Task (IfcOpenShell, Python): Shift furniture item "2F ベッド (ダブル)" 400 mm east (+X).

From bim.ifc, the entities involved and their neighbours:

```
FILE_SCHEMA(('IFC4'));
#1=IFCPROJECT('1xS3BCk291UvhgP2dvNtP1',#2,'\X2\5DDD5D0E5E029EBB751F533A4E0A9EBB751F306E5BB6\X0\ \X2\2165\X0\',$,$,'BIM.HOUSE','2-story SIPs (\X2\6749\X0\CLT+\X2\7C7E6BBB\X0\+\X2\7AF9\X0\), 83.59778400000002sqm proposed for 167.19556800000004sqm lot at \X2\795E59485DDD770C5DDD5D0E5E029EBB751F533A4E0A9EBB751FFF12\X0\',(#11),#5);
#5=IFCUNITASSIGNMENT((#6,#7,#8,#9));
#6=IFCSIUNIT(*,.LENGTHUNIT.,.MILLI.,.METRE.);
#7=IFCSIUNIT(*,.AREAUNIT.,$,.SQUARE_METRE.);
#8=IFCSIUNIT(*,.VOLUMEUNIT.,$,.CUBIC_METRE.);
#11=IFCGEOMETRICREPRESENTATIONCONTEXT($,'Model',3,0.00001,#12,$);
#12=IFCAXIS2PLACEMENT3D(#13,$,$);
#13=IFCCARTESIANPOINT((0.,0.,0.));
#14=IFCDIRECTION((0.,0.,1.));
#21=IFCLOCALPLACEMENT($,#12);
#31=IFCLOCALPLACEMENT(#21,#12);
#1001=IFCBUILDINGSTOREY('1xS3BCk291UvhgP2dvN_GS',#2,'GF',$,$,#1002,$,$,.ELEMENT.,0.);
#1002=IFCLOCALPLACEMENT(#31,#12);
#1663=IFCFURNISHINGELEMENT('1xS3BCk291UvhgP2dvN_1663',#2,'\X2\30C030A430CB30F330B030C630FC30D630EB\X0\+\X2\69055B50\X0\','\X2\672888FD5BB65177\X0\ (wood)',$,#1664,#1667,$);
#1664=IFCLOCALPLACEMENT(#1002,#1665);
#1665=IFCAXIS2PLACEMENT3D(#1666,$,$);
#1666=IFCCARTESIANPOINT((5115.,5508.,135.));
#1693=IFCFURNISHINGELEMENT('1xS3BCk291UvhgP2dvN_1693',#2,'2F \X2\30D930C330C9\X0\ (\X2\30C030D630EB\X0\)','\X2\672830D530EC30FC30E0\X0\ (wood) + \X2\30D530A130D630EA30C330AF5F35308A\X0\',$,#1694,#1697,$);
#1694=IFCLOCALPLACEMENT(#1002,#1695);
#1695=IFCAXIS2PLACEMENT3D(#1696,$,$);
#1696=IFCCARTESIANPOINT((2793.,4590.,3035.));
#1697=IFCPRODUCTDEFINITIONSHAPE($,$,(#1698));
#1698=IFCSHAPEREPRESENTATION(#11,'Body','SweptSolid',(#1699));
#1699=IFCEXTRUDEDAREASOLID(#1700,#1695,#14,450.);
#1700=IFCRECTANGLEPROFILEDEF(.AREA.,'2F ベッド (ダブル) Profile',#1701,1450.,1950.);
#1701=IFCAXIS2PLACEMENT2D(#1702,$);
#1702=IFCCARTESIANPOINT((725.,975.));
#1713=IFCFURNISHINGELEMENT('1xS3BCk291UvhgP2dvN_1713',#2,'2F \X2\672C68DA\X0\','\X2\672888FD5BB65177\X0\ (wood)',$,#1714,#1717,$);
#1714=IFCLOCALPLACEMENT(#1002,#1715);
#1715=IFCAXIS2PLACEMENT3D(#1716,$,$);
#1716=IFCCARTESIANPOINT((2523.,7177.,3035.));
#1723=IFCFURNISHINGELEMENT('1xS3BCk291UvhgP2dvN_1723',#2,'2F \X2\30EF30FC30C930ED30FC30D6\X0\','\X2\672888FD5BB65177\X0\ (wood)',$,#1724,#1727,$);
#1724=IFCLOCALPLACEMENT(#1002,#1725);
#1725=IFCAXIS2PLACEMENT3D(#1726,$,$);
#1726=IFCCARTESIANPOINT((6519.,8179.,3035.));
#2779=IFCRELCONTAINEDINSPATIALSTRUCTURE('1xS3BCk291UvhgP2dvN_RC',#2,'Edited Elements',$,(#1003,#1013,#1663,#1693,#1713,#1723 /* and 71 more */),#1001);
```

```python
import ifcopenshell
import ifcopenshell.api.geometry
import ifcopenshell.util.placement
import ifcopenshell.util.unit

model = ifcopenshell.open("bim.ifc")
unit_scale = ifcopenshell.util.unit.calculate_unit_scale(model)

item = model.by_guid("1xS3BCk291UvhgP2dvN_1693")
matrix = ifcopenshell.util.placement.get_local_placement(item.ObjectPlacement)
matrix[0, 3] += 0.4 / unit_scale
ifcopenshell.api.geometry.edit_object_placement(model, product=item, matrix=matrix, is_si=False)

print(ifcopenshell.util.placement.get_local_placement(item.ObjectPlacement).round(3) + 0.0)

model.write("bim_edited.ifc")
```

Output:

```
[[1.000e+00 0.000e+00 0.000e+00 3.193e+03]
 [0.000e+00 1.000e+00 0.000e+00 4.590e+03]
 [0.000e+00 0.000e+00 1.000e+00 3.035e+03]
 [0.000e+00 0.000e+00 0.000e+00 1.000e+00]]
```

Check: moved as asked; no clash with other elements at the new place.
